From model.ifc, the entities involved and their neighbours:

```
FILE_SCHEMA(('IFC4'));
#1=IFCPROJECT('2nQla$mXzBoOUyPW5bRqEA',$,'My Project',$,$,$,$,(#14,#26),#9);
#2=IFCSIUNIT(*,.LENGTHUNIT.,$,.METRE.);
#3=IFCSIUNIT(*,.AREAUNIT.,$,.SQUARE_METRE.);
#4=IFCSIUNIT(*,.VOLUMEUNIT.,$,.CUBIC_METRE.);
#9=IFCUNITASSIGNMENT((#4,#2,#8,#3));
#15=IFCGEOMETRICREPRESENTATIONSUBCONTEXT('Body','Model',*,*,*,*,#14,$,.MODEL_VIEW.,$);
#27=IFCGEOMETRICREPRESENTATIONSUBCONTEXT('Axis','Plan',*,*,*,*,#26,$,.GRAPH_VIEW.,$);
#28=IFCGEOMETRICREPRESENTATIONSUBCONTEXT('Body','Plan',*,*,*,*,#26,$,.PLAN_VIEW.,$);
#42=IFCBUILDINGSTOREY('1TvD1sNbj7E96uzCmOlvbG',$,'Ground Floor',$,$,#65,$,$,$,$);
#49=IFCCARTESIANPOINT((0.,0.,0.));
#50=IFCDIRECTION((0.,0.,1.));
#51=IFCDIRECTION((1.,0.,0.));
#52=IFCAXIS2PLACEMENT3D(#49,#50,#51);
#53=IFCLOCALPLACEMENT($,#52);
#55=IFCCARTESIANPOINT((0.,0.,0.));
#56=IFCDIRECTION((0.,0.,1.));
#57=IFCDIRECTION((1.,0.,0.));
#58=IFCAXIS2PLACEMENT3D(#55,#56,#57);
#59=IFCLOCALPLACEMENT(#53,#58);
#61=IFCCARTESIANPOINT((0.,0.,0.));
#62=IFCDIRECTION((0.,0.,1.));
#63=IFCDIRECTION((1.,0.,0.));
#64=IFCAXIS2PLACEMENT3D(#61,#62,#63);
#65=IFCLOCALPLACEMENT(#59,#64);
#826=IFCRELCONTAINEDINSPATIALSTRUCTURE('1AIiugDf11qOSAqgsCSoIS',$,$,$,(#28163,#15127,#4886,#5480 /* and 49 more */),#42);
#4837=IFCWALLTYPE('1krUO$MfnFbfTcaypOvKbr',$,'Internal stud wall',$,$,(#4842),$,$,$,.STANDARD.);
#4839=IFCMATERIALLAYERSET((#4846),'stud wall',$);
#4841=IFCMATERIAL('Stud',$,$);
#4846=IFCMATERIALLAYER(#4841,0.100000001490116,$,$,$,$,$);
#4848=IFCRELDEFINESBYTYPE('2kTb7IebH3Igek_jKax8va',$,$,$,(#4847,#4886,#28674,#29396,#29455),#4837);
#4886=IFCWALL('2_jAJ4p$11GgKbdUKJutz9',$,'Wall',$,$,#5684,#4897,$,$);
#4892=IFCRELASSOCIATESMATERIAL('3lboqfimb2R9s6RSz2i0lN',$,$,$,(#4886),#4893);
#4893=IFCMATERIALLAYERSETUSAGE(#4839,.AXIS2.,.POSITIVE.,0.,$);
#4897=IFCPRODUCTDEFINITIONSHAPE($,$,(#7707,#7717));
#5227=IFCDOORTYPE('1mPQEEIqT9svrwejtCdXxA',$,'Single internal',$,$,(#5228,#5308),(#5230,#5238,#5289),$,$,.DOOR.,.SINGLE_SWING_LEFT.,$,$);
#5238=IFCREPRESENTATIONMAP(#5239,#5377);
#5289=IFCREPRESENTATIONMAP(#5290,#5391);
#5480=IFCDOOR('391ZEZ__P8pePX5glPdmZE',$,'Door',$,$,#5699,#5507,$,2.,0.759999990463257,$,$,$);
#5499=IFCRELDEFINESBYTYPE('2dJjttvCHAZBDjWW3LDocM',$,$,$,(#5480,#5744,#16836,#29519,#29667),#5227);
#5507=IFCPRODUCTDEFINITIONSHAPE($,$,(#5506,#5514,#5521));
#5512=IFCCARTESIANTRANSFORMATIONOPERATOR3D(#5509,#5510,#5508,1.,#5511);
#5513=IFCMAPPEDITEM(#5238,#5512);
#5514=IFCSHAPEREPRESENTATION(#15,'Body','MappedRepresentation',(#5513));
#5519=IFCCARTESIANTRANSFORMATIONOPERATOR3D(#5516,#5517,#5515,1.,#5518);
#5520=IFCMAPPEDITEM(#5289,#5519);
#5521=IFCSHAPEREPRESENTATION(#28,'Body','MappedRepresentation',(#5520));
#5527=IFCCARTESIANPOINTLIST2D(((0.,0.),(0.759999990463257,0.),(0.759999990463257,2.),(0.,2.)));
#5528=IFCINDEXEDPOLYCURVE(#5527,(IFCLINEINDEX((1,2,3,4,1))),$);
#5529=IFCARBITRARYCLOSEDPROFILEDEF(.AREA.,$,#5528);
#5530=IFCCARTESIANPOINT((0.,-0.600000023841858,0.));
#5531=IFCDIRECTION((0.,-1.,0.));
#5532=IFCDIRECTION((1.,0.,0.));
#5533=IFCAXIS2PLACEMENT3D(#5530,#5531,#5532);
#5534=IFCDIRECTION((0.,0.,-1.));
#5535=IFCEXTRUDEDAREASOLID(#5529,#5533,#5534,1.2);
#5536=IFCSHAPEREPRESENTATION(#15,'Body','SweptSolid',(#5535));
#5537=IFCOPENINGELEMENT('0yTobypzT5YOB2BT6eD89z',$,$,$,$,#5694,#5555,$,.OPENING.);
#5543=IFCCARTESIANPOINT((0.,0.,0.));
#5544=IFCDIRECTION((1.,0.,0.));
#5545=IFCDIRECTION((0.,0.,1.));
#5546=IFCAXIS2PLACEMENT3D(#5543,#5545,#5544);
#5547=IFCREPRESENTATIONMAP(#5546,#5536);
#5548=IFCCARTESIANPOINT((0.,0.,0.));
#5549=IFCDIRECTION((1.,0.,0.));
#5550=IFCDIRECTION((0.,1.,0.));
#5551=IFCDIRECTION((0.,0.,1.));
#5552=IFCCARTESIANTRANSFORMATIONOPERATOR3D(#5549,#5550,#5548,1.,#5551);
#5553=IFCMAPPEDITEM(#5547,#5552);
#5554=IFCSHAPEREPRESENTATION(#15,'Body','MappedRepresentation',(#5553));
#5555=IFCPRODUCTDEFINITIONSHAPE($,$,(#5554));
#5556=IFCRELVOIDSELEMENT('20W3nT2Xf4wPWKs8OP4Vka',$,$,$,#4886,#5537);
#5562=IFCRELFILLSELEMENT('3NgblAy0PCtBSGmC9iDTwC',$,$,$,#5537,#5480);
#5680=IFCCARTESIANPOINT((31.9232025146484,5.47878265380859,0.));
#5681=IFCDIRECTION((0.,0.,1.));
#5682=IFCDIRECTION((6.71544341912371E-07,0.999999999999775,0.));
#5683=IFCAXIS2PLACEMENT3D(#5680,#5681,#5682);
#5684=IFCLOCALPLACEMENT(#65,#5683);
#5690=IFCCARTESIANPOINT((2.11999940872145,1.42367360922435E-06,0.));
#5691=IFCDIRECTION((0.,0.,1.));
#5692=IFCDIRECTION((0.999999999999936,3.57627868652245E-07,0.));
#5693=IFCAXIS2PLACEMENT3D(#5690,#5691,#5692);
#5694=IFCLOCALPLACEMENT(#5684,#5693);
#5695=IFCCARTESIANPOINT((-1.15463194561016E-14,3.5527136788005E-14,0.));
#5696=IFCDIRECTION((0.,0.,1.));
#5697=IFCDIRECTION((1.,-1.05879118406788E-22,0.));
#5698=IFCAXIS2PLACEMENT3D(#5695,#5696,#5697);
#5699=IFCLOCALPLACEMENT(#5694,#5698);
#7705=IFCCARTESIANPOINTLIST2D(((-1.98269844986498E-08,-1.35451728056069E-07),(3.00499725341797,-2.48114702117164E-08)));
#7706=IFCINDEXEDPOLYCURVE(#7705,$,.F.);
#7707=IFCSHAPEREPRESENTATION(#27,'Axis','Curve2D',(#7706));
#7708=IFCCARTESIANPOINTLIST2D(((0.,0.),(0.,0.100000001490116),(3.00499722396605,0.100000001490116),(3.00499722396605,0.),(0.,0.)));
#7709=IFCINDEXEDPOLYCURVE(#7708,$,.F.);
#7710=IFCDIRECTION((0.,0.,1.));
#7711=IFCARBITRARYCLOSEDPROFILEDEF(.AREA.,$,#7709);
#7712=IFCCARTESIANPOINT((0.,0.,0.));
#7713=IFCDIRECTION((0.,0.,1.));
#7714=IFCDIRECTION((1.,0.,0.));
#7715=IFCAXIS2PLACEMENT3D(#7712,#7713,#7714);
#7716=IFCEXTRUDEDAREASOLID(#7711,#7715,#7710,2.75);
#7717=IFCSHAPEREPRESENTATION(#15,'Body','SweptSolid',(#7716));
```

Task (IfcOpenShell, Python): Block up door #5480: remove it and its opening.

```python
import ifcopenshell
import ifcopenshell.api.feature
import ifcopenshell.api.root
import ifcopenshell.geom
import ifcopenshell.util.shape

model = ifcopenshell.open("model.ifc")
settings = ifcopenshell.geom.settings()


def volume(element):
    """Net volume in cubic metres, openings subtracted."""
    shape = ifcopenshell.geom.create_shape(settings, element)
    return ifcopenshell.util.shape.get_volume(shape.geometry)


door = model.by_guid("391ZEZ__P8pePX5glPdmZE")
opening = door.FillsVoids[0].RelatingOpeningElement
wall = opening.VoidsElements[0].RelatingBuildingElement
before = volume(wall)

ifcopenshell.api.root.remove_product(model, product=door)
ifcopenshell.api.feature.remove_feature(model, feature=opening)

after = volume(wall)

print(f"wall volume {before:.3f} -> {after:.3f} m3")

model.write("model_v2.ifc")
```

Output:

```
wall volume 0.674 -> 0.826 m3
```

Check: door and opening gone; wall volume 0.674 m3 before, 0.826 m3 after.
